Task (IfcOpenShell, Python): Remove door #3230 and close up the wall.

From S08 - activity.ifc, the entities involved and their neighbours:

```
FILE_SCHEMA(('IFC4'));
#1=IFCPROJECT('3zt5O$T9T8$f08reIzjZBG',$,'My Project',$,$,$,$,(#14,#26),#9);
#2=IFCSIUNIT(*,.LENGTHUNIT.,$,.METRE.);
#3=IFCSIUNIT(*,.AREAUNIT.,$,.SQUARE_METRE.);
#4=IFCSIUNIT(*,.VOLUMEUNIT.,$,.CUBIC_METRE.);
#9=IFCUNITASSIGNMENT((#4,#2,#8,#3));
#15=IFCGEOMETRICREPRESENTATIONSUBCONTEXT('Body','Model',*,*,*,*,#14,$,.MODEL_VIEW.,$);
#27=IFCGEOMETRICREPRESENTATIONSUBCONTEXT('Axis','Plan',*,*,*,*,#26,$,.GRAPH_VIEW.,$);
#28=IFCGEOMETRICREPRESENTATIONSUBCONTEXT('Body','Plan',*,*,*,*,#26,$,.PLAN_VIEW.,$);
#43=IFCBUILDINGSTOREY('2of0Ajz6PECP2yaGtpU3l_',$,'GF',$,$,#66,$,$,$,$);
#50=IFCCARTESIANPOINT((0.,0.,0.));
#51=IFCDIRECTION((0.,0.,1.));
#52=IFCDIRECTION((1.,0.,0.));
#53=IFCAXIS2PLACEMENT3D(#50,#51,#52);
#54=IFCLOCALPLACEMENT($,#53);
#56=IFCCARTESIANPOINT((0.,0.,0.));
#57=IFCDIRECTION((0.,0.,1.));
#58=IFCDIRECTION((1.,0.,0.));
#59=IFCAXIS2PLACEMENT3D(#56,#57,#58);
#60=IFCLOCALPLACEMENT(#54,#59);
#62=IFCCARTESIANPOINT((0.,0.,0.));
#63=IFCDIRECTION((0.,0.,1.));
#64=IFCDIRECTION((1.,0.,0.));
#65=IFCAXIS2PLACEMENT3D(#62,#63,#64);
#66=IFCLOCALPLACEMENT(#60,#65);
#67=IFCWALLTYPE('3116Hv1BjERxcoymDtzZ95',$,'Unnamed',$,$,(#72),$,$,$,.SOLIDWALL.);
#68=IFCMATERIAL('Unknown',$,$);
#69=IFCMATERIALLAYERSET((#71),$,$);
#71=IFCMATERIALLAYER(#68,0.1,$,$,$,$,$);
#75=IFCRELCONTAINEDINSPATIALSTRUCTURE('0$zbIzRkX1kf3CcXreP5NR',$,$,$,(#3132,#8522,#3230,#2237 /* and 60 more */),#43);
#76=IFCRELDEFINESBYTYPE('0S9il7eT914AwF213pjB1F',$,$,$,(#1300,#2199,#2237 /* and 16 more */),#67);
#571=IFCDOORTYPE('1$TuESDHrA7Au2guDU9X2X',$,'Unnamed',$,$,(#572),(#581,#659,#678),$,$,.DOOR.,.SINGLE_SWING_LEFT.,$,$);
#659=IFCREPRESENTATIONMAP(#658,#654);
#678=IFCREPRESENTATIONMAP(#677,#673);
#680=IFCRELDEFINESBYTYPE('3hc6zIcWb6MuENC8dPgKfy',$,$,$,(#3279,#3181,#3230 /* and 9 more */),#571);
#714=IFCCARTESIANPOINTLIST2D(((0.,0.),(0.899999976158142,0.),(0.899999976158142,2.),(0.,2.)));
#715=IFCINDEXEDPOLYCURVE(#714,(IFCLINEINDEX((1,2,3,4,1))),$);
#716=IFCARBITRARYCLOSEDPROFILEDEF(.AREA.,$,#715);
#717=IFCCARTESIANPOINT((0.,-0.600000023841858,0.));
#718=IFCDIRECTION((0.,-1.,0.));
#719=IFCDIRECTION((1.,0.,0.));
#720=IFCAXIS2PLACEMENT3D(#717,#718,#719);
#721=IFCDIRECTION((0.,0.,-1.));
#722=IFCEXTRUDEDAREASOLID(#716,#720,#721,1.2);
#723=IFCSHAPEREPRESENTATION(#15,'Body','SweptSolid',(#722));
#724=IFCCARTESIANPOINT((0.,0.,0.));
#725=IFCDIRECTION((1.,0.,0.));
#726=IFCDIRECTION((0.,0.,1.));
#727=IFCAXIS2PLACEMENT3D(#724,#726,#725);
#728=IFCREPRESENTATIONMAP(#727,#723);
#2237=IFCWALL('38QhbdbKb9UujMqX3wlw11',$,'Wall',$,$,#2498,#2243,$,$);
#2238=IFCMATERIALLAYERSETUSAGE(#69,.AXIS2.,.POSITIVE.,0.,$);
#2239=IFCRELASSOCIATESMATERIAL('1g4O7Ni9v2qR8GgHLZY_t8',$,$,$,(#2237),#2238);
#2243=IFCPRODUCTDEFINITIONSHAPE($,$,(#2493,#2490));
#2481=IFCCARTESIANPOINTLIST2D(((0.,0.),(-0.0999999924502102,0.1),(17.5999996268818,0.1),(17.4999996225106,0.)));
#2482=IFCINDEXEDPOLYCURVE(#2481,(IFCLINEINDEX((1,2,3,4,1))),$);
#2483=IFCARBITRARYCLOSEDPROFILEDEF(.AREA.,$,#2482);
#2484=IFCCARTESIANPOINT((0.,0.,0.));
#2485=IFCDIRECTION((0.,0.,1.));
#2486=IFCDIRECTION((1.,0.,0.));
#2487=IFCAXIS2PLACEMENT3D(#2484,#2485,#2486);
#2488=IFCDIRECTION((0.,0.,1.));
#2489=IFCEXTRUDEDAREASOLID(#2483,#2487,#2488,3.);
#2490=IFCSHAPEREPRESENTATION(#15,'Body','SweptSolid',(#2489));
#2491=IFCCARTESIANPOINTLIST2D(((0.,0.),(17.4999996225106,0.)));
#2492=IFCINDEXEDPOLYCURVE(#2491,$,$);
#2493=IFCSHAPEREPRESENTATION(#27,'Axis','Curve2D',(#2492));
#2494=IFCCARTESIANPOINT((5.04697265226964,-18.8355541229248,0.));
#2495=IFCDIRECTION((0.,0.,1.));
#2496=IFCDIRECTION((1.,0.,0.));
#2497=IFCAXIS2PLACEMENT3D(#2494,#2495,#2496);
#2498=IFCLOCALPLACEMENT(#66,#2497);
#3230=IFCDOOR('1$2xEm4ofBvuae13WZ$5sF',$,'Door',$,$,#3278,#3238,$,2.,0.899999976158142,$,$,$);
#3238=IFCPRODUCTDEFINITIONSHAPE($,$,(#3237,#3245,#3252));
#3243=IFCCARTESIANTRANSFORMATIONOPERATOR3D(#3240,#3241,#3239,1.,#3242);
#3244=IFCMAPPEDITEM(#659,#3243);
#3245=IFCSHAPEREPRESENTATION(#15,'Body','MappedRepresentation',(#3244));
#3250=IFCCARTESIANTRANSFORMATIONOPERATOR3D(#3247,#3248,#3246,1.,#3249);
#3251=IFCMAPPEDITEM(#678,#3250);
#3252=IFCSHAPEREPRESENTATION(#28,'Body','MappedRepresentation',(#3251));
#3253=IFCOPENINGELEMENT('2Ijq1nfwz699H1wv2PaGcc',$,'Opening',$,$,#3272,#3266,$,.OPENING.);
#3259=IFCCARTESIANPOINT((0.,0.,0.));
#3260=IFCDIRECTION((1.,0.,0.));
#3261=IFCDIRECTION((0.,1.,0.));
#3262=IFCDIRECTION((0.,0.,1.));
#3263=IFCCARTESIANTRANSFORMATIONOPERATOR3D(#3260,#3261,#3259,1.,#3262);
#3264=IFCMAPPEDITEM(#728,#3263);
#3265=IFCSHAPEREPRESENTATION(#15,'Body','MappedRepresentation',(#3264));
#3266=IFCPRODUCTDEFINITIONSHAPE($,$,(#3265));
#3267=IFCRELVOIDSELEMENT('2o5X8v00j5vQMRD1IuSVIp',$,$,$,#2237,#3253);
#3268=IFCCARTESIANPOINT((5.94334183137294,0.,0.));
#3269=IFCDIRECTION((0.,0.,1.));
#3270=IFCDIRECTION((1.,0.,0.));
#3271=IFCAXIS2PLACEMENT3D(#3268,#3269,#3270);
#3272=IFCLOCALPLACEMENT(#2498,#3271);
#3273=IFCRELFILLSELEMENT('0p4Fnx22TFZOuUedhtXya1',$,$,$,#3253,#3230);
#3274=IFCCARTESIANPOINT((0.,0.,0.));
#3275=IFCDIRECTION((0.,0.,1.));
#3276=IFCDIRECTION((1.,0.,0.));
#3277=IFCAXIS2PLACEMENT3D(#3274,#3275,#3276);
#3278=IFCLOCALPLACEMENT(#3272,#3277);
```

```python
import ifcopenshell
import ifcopenshell.api.feature
import ifcopenshell.api.root
import ifcopenshell.geom
import ifcopenshell.util.shape

model = ifcopenshell.open("S08 - activity.ifc")
settings = ifcopenshell.geom.settings()


def volume(element):
    """Net volume in cubic metres, openings subtracted."""
    shape = ifcopenshell.geom.create_shape(settings, element)
    return ifcopenshell.util.shape.get_volume(shape.geometry)


door = model.by_guid("1$2xEm4ofBvuae13WZ$5sF")
opening = door.FillsVoids[0].RelatingOpeningElement
wall = opening.VoidsElements[0].RelatingBuildingElement
before = volume(wall)

ifcopenshell.api.root.remove_product(model, product=door)
ifcopenshell.api.feature.remove_feature(model, feature=opening)

after = volume(wall)

print(f"wall volume {before:.3f} -> {after:.3f} m3")

model.write("S08 - activity_rev.ifc")
```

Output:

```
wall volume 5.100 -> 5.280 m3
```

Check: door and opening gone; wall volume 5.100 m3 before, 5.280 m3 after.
